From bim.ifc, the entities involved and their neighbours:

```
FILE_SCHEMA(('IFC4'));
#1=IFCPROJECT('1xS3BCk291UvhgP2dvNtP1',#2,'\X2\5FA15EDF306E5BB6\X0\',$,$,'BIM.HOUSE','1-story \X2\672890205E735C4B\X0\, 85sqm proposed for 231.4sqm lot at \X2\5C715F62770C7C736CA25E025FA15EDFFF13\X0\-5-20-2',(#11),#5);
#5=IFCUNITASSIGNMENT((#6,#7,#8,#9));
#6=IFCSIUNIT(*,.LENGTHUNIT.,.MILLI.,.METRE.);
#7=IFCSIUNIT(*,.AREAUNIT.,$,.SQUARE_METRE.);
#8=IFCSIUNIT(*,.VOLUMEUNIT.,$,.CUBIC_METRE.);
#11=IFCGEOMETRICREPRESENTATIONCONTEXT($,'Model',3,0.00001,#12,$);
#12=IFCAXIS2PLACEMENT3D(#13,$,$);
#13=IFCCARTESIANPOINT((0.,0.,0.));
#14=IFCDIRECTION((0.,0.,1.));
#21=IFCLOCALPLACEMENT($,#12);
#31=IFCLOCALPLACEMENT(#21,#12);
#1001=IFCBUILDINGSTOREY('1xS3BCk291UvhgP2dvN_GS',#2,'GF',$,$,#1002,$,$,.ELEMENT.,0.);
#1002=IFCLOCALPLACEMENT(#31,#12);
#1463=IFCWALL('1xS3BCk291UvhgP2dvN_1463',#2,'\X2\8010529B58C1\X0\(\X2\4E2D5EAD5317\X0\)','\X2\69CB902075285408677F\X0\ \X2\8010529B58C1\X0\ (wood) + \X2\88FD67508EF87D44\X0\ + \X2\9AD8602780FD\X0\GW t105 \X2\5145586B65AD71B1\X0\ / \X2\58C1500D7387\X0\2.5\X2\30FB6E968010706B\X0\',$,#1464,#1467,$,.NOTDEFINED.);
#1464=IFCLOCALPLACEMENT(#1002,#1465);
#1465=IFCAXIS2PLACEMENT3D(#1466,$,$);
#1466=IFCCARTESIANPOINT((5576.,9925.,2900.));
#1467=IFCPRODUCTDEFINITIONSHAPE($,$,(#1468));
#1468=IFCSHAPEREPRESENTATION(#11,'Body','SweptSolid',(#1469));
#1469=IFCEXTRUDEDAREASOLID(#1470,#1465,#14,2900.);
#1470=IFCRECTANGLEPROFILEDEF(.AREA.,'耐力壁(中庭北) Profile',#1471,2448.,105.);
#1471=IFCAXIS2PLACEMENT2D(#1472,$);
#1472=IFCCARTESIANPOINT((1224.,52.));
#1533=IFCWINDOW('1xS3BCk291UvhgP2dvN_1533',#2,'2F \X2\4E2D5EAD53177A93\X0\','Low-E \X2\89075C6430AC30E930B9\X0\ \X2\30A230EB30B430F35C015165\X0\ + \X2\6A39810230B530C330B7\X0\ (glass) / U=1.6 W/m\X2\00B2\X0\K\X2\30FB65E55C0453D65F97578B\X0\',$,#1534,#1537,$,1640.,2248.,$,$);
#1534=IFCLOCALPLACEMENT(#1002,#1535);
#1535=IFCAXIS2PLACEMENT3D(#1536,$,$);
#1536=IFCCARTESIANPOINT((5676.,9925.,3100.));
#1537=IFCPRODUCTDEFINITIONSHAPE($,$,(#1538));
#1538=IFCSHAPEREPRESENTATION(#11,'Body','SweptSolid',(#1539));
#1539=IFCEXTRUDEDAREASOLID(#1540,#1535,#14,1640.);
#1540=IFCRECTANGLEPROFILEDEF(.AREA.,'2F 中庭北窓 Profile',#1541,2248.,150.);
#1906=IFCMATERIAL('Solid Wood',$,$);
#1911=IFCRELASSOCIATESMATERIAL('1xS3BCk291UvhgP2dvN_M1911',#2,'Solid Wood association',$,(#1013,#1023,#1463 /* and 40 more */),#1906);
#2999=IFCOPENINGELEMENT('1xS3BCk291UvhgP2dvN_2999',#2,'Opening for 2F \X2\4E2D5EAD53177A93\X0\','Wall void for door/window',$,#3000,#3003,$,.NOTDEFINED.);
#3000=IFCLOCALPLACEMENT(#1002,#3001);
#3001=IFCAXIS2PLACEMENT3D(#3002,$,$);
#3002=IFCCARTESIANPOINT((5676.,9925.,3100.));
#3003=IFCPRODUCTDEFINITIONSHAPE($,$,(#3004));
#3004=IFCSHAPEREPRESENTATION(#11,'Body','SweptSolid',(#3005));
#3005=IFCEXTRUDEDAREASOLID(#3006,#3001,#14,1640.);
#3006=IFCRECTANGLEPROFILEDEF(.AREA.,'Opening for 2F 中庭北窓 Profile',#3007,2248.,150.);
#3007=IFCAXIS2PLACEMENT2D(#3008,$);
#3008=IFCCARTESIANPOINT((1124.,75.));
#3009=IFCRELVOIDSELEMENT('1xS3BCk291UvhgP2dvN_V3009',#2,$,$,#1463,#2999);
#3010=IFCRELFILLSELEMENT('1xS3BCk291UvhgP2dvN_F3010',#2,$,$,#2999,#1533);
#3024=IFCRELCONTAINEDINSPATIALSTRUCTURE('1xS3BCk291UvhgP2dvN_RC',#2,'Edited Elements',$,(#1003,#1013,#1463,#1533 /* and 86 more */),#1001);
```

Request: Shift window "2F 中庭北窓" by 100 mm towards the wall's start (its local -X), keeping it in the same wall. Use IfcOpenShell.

```python
import ifcopenshell
import ifcopenshell.api.geometry
import ifcopenshell.util.placement
import ifcopenshell.util.unit

model = ifcopenshell.open("bim.ifc")
unit_scale = ifcopenshell.util.unit.calculate_unit_scale(model)

window = model.by_guid("1xS3BCk291UvhgP2dvN_1533")
opening = window.FillsVoids[0].RelatingOpeningElement
wall = opening.VoidsElements[0].RelatingBuildingElement

wall_matrix = ifcopenshell.util.placement.get_local_placement(wall.ObjectPlacement)
shift = wall_matrix[:3, 0] * -0.1 / unit_scale
before = ifcopenshell.util.placement.get_local_placement(window.ObjectPlacement)[:3, 3].copy()

# The window is not placed relative to its opening, so move both.
for product in (opening, window):
    matrix = ifcopenshell.util.placement.get_local_placement(product.ObjectPlacement)
    matrix[:3, 3] += shift
    ifcopenshell.api.geometry.edit_object_placement(model, product=product, matrix=matrix, is_si=False)

after = ifcopenshell.util.placement.get_local_placement(window.ObjectPlacement)[:3, 3]
print("window moved by", (after - before).round(3) + 0.0)

model.write("bim_edited.ifc")
```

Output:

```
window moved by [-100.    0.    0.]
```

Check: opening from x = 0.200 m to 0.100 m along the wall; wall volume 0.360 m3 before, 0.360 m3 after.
